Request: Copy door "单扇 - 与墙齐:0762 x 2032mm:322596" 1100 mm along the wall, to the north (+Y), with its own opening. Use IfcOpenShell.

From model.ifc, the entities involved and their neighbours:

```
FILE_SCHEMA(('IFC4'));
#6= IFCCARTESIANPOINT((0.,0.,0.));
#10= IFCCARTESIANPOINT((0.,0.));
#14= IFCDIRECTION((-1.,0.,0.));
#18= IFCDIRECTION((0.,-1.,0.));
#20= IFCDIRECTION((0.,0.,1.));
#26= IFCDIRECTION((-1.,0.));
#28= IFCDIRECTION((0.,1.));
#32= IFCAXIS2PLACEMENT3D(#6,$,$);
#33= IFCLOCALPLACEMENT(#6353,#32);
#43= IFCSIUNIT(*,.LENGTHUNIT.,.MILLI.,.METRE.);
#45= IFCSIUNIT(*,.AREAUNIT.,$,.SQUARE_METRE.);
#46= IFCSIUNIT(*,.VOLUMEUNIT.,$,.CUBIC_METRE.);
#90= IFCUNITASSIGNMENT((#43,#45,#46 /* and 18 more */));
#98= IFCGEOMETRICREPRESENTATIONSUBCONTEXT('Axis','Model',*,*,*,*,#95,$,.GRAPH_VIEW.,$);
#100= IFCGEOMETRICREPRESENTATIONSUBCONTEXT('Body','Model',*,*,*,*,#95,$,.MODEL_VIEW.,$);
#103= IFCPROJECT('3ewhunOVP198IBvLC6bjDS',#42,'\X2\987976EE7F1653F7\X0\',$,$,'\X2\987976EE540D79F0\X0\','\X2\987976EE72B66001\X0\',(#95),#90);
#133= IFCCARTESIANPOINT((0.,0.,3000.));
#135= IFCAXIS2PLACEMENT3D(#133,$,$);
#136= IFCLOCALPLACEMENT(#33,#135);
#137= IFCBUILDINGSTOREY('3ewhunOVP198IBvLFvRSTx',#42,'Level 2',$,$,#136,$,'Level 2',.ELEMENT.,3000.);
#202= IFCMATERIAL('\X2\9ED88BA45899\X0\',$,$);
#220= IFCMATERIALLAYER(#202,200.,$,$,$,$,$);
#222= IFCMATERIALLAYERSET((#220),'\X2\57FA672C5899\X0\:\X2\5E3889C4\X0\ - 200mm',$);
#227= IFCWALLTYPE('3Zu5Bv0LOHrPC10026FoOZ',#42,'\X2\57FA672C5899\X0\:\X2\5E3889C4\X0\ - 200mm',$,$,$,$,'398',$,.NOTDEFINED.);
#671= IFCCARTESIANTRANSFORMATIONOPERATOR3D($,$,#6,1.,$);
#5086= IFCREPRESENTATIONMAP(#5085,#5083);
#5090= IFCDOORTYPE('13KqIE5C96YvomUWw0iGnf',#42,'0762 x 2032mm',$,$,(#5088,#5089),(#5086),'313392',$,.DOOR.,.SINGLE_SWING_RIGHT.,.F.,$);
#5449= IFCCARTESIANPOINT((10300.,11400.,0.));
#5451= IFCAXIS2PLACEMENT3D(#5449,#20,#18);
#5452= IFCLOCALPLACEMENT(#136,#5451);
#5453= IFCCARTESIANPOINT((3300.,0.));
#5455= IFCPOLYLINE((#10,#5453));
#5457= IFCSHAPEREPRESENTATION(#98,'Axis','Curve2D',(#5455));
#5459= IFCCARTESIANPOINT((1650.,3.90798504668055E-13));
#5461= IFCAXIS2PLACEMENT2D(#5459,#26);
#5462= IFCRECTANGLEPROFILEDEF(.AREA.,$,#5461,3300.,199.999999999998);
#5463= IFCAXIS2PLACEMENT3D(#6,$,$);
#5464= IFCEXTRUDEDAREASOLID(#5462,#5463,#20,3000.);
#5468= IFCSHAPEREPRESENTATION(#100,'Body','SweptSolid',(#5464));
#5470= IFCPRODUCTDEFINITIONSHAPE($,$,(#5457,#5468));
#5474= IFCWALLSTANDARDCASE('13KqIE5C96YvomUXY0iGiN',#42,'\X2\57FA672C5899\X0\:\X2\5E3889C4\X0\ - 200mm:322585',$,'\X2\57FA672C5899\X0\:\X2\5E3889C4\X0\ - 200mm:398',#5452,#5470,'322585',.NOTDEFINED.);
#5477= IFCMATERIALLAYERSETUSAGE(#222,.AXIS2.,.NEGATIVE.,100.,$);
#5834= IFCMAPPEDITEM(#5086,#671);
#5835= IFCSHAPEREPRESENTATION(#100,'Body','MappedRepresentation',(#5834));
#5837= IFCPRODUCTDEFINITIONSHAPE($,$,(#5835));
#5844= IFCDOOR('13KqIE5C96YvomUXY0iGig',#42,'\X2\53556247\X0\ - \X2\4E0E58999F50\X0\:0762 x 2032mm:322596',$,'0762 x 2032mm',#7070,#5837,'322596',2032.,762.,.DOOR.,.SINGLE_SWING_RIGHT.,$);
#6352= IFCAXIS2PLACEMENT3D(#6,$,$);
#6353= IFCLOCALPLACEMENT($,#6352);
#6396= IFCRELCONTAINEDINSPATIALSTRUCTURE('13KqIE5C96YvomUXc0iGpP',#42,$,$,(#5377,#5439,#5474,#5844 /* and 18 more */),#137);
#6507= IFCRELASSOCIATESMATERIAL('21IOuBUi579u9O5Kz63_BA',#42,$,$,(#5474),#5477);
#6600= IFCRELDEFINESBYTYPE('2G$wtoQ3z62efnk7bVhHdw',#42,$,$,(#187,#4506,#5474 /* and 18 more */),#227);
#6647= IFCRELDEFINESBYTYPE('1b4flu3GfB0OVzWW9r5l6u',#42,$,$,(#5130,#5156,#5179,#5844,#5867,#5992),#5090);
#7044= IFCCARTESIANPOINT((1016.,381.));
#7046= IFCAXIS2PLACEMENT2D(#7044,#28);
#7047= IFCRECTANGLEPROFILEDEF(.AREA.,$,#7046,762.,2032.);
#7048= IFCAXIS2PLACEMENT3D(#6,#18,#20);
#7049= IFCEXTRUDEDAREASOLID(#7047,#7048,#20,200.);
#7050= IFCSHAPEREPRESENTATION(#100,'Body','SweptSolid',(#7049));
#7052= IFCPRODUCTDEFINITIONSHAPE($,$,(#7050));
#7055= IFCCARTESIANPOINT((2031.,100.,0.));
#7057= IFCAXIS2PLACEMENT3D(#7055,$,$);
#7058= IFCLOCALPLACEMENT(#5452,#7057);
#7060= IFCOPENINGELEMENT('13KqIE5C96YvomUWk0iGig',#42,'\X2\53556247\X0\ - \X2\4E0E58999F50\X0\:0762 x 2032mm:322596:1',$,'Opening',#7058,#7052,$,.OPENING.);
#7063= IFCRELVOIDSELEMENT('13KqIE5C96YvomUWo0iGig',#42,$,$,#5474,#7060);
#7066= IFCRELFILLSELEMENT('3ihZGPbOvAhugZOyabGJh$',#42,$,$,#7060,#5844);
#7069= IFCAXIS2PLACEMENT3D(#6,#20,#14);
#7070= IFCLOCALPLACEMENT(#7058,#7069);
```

```python
import ifcopenshell
import ifcopenshell.api.feature
import ifcopenshell.api.geometry
import ifcopenshell.api.root
import ifcopenshell.geom
import ifcopenshell.util.element
import ifcopenshell.util.placement
import ifcopenshell.util.shape
import ifcopenshell.util.unit

model = ifcopenshell.open("model.ifc")
unit_scale = ifcopenshell.util.unit.calculate_unit_scale(model)
settings = ifcopenshell.geom.settings()


def volume(element):
    """Net volume in cubic metres, openings subtracted."""
    shape = ifcopenshell.geom.create_shape(settings, element)
    return ifcopenshell.util.shape.get_volume(shape.geometry)


def reuse_history(source, copy):
    """copy_class also copies each property set's owner history, people and application; keep the originals."""
    for rel in copy.IsDefinedBy:
        if rel.is_a("IfcRelDefinesByProperties") and (history := rel.RelatingPropertyDefinition.OwnerHistory):
            rel.RelatingPropertyDefinition.OwnerHistory = source.OwnerHistory
            ifcopenshell.util.element.remove_deep2(model, history)


door = model.by_guid("13KqIE5C96YvomUXY0iGig")
opening = door.FillsVoids[0].RelatingOpeningElement
wall = opening.VoidsElements[0].RelatingBuildingElement
before = volume(wall)
shift = ifcopenshell.util.placement.get_local_placement(wall.ObjectPlacement)[:3, 0] * -1.1 / unit_scale

# copy_class copies the void relationship, type, container and properties, but no geometry.
new_opening = ifcopenshell.api.root.copy_class(model, product=opening)
new_opening.Representation = ifcopenshell.util.element.copy_deep(
    model, opening.Representation, exclude=["IfcGeometricRepresentationContext", "IfcRepresentationMap"]
)
new_opening.Name = "单扇 - 与墙齐:0762 x 2032mm"
new_door = ifcopenshell.api.root.copy_class(model, product=door)
new_door.Representation = ifcopenshell.util.element.copy_deep(
    model, door.Representation, exclude=["IfcGeometricRepresentationContext", "IfcRepresentationMap"]
)
new_door.Name = "单扇 - 与墙齐:0762 x 2032mm"
new_door.Tag = None
reuse_history(door, new_door)
ifcopenshell.api.feature.add_filling(model, opening=new_opening, element=new_door)

for old, new in ((opening, new_opening), (door, new_door)):
    matrix = ifcopenshell.util.placement.get_local_placement(old.ObjectPlacement)
    matrix[:3, 3] += shift
    ifcopenshell.api.geometry.edit_object_placement(model, product=new, matrix=matrix, is_si=False)

after = volume(wall)

print(f"wall volume {before:.3f} -> {after:.3f} m3")

model.write("model_edited.ifc")
```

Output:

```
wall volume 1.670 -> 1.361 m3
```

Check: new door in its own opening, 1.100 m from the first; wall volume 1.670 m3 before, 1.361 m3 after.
